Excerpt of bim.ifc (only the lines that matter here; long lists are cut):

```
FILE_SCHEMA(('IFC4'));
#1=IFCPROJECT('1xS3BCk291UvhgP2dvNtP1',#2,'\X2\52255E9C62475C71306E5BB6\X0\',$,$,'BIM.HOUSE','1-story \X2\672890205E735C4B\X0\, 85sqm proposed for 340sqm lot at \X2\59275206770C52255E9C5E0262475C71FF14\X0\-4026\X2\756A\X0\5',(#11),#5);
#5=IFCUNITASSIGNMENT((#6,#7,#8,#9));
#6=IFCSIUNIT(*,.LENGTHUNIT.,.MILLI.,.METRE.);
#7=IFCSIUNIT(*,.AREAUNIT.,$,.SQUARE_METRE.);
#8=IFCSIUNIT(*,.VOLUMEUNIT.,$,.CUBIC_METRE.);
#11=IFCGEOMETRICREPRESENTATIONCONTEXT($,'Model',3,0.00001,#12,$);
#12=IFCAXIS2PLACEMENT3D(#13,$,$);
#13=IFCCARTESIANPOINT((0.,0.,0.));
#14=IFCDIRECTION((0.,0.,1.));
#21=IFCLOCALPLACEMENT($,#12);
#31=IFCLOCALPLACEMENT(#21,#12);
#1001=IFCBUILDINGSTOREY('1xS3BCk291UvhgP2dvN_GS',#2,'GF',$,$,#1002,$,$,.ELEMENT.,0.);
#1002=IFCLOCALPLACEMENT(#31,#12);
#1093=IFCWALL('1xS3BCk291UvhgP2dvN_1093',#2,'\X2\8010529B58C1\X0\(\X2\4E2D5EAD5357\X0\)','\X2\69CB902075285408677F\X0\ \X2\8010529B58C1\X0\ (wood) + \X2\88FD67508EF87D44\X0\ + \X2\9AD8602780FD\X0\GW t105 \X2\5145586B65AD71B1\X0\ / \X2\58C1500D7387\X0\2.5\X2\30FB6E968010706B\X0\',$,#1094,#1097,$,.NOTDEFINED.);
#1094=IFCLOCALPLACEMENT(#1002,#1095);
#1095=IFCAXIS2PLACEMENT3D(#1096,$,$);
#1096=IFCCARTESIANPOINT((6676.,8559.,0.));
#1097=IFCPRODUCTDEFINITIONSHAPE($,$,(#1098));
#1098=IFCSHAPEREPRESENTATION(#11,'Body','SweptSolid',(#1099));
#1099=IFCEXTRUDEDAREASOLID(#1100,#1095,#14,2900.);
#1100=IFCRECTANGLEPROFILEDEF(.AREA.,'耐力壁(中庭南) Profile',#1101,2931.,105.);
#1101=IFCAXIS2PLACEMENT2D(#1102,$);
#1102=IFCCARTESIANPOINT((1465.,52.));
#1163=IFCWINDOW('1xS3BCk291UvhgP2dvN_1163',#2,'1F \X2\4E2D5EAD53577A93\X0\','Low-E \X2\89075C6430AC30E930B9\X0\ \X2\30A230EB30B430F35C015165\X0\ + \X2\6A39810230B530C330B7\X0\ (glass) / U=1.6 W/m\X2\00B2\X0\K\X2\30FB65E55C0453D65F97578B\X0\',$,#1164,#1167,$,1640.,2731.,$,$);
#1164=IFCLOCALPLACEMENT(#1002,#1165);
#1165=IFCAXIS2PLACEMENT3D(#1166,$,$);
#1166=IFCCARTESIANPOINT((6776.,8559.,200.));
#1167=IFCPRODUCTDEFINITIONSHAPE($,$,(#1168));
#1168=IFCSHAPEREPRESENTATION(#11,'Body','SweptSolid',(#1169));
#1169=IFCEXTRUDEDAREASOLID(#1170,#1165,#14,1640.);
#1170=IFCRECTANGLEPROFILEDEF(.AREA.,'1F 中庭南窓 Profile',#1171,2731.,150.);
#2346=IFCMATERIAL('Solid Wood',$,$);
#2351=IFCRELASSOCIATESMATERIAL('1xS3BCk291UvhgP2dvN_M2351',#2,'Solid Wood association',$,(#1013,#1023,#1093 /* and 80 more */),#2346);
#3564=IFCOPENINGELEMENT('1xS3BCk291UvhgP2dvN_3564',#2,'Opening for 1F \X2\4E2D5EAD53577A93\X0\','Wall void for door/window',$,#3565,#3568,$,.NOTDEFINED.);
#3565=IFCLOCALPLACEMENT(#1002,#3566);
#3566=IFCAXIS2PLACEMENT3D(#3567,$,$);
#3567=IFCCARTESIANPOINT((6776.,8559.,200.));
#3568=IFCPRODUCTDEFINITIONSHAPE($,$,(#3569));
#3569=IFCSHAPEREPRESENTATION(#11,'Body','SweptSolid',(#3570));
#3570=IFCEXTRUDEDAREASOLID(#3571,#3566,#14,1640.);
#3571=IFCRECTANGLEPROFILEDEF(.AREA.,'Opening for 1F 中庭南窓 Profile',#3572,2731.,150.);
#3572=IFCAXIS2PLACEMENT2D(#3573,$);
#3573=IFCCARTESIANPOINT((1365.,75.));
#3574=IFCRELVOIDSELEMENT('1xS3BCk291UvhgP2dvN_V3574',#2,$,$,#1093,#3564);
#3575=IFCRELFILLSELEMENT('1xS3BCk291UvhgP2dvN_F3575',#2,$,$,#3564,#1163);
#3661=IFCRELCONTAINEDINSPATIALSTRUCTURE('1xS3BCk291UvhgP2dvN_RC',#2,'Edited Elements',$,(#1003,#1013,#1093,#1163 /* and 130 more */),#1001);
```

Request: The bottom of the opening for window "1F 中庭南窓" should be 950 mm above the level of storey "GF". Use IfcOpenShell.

```python
import numpy as np
import ifcopenshell
import ifcopenshell.api.geometry
import ifcopenshell.geom
import ifcopenshell.util.element
import ifcopenshell.util.placement
import ifcopenshell.util.shape
import ifcopenshell.util.unit

model = ifcopenshell.open("bim.ifc")
unit_scale = ifcopenshell.util.unit.calculate_unit_scale(model)

window = model.by_guid("1xS3BCk291UvhgP2dvN_1163")
opening = window.FillsVoids[0].RelatingOpeningElement
storey = ifcopenshell.util.element.get_container(window, ifc_class="IfcBuildingStorey")
level = ifcopenshell.util.placement.get_local_placement(storey.ObjectPlacement)[2, 3]

# The opening's origin need not be at the sill, so measure its lowest point.
shape = ifcopenshell.geom.create_shape(ifcopenshell.geom.settings(), opening)
bottom = ifcopenshell.util.shape.get_shape_bottom_elevation(shape, shape.geometry) / unit_scale
dz = level + 0.95 / unit_scale - bottom

shift = np.array([0.0, 0.0, dz])
# The window is not placed relative to its opening, so move both.
for product in (opening, window):
    matrix = ifcopenshell.util.placement.get_local_placement(product.ObjectPlacement)
    matrix[:3, 3] += shift
    ifcopenshell.api.geometry.edit_object_placement(model, product=product, matrix=matrix, is_si=False)

print(f"moved by {dz * unit_scale:+.3f} m")

model.write("bim_updated.ifc")
```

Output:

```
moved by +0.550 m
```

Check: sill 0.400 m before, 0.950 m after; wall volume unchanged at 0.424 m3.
